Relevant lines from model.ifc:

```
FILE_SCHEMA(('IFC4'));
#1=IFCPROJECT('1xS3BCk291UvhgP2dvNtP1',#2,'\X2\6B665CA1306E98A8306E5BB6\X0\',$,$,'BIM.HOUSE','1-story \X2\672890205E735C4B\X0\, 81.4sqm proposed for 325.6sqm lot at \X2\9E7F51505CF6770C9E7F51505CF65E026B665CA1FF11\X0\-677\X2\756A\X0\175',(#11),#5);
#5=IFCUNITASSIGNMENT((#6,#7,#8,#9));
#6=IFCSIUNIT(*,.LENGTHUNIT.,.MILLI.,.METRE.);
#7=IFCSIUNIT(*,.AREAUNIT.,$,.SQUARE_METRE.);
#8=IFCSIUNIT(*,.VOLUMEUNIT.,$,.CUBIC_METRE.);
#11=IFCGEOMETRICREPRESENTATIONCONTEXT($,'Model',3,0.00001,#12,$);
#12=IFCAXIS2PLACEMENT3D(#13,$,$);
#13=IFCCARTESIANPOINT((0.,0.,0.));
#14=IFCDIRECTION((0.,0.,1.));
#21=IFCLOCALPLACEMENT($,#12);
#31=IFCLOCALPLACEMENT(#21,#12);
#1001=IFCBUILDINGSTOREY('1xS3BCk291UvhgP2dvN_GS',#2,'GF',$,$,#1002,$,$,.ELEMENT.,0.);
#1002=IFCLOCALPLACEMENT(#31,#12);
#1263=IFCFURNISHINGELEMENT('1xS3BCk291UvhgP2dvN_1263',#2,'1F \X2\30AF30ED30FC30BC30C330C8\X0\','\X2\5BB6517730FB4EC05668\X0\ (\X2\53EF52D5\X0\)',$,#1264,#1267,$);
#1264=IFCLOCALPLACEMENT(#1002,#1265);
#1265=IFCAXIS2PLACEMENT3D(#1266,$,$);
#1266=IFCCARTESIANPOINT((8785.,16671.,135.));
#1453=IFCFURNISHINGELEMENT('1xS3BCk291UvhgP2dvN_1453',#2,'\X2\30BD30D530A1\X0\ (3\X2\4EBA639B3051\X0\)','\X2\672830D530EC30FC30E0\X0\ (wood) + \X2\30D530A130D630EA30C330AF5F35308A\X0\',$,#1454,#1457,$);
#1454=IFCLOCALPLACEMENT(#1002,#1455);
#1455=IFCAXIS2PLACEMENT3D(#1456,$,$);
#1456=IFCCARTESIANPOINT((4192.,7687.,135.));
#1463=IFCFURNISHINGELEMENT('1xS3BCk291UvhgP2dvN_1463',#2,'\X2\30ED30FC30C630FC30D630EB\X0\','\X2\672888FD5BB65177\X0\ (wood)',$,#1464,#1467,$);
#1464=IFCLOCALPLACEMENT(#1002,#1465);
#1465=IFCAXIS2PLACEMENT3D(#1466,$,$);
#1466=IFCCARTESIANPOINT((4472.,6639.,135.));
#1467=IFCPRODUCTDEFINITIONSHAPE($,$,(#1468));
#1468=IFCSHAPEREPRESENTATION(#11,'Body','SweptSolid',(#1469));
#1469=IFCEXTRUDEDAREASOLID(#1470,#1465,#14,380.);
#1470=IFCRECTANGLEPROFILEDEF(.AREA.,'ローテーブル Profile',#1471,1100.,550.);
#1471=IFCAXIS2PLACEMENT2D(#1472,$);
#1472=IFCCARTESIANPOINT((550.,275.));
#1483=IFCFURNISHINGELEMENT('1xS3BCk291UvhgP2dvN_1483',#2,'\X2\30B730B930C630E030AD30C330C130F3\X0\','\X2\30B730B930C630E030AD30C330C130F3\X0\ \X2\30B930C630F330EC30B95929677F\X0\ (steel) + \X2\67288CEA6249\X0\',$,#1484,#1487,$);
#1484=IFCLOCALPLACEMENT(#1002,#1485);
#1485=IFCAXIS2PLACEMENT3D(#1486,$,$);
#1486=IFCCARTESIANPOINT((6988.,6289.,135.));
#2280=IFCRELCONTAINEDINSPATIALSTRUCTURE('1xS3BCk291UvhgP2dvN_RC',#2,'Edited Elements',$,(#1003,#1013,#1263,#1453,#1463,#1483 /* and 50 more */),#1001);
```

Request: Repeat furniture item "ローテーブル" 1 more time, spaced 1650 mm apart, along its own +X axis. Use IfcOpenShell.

```python
import ifcopenshell
import ifcopenshell.api.geometry
import ifcopenshell.api.root
import ifcopenshell.util.element
import ifcopenshell.util.placement
import ifcopenshell.util.unit

model = ifcopenshell.open("model.ifc")
unit_scale = ifcopenshell.util.unit.calculate_unit_scale(model)


def reuse_history(source, copy):
    """copy_class also copies each property set's owner history, people and application; keep the originals."""
    for rel in copy.IsDefinedBy:
        if rel.is_a("IfcRelDefinesByProperties") and (history := rel.RelatingPropertyDefinition.OwnerHistory):
            rel.RelatingPropertyDefinition.OwnerHistory = source.OwnerHistory
            ifcopenshell.util.element.remove_deep2(model, history)


source = model.by_guid("1xS3BCk291UvhgP2dvN_1463")
base = ifcopenshell.util.placement.get_local_placement(source.ObjectPlacement)
step = base[:3, 0] * 1.65 / unit_scale

for i in range(1, 2):
    copy = ifcopenshell.api.root.copy_class(model, product=source)
    copy.Representation = ifcopenshell.util.element.copy_deep(
        model, source.Representation, exclude=["IfcGeometricRepresentationContext", "IfcRepresentationMap"]
    )
    reuse_history(source, copy)
    matrix = base.copy()
    matrix[:3, 3] += i * step
    print("added at", matrix[:3, 3].round(3) + 0.0)
    ifcopenshell.api.geometry.edit_object_placement(model, product=copy, matrix=matrix, is_si=False)

model.write("model_edited.ifc")
```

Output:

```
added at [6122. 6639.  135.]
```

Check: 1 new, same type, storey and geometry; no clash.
